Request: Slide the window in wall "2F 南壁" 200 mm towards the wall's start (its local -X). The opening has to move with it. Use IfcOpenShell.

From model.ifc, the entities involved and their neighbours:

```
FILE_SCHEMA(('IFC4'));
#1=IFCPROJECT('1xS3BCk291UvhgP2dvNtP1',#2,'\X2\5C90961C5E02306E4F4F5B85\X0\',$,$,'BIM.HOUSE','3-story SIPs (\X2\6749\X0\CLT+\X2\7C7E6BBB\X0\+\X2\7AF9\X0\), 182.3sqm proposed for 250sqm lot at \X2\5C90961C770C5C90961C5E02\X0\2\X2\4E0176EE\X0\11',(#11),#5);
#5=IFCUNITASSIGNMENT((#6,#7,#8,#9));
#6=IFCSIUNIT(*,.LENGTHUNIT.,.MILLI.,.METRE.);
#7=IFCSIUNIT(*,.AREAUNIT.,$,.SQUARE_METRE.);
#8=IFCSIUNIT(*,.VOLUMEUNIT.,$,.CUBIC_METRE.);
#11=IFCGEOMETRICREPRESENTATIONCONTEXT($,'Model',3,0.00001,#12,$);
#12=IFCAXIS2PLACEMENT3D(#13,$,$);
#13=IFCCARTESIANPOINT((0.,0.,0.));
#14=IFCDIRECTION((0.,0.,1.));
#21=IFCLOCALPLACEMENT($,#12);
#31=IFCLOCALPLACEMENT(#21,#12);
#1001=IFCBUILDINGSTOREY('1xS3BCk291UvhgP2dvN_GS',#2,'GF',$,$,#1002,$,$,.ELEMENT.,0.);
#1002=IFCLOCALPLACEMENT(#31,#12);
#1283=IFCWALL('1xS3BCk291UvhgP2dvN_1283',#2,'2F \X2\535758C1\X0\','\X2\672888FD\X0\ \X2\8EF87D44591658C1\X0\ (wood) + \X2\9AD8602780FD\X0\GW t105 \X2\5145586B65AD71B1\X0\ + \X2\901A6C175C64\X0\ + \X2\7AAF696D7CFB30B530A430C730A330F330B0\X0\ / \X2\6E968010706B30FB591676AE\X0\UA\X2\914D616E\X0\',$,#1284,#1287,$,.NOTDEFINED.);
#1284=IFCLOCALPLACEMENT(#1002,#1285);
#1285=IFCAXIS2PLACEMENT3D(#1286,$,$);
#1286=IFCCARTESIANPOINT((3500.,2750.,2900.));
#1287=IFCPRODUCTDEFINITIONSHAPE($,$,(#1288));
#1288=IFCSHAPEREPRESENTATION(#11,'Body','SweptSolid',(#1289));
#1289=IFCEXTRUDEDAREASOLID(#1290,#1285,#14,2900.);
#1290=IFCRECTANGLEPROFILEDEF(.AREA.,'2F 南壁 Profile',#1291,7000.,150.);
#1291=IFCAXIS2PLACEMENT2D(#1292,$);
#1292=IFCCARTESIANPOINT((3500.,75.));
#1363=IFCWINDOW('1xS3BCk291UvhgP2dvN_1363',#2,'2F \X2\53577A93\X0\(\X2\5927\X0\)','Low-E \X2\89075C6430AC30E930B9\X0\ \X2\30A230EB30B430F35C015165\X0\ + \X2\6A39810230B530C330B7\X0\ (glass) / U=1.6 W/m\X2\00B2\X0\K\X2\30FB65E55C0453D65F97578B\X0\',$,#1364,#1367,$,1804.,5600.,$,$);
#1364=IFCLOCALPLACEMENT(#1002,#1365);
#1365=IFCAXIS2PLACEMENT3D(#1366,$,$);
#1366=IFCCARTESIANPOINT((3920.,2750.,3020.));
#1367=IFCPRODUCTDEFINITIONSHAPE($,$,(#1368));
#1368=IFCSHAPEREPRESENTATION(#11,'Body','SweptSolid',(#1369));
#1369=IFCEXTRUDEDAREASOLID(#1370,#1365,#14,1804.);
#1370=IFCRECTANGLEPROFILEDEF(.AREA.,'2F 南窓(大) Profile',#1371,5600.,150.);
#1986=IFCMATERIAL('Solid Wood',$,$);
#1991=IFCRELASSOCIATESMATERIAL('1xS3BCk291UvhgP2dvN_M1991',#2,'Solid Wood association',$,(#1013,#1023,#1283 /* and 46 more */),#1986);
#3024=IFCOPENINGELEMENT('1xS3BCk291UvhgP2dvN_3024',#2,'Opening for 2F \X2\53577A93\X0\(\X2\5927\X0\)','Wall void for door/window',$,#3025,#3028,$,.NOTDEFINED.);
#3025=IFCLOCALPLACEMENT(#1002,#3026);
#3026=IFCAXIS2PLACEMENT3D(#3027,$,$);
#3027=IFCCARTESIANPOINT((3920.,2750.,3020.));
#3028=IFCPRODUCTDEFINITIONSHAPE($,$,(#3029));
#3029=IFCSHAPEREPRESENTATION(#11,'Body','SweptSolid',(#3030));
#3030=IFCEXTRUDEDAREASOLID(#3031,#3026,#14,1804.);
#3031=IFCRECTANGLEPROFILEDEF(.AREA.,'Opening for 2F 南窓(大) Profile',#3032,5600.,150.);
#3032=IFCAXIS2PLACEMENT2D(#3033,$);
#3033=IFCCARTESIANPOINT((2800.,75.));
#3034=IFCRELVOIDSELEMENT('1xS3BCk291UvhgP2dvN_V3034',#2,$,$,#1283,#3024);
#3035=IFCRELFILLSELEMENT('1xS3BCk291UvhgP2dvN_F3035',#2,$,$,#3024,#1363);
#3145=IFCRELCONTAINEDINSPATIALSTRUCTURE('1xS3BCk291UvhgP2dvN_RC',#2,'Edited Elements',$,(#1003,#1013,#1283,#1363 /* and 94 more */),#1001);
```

```python
import ifcopenshell
import ifcopenshell.api.geometry
import ifcopenshell.util.placement

model = ifcopenshell.open("model.ifc")

window = model.by_id(1363)
opening = window.FillsVoids[0].RelatingOpeningElement
wall = opening.VoidsElements[0].RelatingBuildingElement

wall_matrix = ifcopenshell.util.placement.get_local_placement(wall.ObjectPlacement)
shift = wall_matrix[:3, 0] * -200.0
before = ifcopenshell.util.placement.get_local_placement(window.ObjectPlacement)[:3, 3].copy()

# The window is not placed relative to its opening, so move both.
for product in (opening, window):
    matrix = ifcopenshell.util.placement.get_local_placement(product.ObjectPlacement)
    matrix[:3, 3] += shift
    ifcopenshell.api.geometry.edit_object_placement(model, product=product, matrix=matrix, is_si=False)

after = ifcopenshell.util.placement.get_local_placement(window.ObjectPlacement)[:3, 3]
print("window moved by", (after - before).round(3) + 0.0)

model.write("model_v2.ifc")
```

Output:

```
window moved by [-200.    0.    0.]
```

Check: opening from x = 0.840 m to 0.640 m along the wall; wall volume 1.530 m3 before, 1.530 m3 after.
